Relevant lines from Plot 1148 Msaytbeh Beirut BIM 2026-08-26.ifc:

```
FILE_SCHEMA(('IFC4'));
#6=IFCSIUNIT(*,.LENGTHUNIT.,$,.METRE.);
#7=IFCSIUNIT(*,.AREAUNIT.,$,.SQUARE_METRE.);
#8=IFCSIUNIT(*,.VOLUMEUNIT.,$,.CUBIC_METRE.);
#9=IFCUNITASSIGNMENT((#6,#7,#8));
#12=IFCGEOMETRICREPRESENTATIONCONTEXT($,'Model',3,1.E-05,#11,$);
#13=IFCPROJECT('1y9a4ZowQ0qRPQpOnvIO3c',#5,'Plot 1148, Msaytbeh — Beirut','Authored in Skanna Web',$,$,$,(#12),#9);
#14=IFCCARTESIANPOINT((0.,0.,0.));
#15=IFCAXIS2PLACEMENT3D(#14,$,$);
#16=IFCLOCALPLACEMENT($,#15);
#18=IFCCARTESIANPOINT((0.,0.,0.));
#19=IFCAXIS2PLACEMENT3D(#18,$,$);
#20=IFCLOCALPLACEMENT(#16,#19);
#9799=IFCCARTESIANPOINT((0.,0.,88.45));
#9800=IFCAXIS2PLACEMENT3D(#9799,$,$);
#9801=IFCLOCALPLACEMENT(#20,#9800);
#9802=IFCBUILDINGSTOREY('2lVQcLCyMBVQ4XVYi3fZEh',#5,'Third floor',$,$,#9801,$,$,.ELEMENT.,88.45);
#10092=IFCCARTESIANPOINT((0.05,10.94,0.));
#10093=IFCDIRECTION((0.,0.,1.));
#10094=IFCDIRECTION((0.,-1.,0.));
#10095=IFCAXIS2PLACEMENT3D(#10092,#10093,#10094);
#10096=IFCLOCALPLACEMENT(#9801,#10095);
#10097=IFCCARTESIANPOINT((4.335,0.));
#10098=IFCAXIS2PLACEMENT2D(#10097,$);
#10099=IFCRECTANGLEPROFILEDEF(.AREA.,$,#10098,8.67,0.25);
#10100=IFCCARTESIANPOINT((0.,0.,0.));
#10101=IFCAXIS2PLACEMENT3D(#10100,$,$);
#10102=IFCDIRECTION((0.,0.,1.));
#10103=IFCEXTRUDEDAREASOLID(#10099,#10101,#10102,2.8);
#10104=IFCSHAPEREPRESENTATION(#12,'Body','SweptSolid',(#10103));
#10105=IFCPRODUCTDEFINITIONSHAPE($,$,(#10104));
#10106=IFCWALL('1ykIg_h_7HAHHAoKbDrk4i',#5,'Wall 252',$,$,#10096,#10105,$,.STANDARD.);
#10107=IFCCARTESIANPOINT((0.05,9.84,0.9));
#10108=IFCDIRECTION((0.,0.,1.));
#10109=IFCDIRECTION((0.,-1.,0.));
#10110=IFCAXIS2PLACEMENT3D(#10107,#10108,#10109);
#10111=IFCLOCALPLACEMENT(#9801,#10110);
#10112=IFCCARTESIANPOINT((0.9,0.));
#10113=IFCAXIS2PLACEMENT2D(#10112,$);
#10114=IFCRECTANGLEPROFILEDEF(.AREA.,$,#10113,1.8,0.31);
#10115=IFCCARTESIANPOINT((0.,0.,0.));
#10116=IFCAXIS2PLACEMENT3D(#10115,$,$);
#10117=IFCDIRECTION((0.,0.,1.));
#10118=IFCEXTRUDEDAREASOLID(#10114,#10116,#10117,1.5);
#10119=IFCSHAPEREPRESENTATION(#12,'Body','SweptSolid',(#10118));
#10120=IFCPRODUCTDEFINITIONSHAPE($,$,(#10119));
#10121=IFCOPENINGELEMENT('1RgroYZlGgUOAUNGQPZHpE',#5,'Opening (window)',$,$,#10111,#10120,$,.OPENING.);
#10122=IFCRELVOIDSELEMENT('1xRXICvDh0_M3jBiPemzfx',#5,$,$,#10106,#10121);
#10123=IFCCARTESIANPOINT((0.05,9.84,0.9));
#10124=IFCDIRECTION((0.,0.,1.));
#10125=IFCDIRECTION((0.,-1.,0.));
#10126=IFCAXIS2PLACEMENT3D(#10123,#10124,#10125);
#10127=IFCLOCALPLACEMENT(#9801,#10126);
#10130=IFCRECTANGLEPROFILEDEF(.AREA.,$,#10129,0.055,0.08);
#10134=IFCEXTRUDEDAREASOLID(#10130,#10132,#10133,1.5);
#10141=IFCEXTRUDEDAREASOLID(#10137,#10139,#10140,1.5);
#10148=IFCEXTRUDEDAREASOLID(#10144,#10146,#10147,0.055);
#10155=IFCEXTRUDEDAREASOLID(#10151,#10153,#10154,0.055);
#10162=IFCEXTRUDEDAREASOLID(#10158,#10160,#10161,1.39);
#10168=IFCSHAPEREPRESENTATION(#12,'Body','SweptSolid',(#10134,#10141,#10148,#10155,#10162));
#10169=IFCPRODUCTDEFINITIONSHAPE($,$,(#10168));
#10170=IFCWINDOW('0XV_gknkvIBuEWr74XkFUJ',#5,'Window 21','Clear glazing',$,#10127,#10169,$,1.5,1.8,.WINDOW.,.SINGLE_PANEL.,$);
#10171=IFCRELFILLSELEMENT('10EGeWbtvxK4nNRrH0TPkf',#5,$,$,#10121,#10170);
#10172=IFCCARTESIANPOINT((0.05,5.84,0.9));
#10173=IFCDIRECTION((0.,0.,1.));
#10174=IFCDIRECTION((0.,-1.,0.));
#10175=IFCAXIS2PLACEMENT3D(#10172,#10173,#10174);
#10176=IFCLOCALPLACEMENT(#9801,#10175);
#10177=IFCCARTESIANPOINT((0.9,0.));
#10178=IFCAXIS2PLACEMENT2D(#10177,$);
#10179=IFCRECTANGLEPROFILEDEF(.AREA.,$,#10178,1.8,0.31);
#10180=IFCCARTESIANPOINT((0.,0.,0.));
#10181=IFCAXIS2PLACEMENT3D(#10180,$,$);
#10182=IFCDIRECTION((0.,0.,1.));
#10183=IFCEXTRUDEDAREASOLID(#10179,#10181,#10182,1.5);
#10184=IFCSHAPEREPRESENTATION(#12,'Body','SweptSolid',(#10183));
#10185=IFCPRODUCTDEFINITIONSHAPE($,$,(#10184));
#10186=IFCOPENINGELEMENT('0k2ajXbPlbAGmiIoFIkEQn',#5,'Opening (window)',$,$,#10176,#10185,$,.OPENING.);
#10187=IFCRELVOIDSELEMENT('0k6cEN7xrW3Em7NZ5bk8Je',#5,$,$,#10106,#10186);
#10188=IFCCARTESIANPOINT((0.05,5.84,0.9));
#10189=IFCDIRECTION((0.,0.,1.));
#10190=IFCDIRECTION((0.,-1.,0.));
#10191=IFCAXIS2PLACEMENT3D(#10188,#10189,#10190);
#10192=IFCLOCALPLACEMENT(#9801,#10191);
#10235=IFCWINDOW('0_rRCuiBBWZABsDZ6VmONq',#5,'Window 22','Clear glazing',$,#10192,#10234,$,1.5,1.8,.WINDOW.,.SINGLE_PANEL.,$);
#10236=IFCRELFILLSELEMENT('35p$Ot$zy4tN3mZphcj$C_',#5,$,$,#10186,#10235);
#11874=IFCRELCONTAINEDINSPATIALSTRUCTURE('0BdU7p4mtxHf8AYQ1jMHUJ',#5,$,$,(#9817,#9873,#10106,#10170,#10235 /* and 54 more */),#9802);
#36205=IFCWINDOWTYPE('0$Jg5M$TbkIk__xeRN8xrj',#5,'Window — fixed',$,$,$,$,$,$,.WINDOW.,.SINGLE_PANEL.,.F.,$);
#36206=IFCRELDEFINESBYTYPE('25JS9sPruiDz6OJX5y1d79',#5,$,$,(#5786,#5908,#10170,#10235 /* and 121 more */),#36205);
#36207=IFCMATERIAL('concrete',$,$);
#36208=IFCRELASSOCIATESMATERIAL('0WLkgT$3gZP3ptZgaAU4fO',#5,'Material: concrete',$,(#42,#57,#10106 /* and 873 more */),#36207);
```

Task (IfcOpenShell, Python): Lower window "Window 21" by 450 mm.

```python
import numpy as np
import ifcopenshell
import ifcopenshell.api.geometry
import ifcopenshell.util.placement
import ifcopenshell.util.unit

model = ifcopenshell.open("Plot 1148 Msaytbeh Beirut BIM 2026-08-26.ifc")
unit_scale = ifcopenshell.util.unit.calculate_unit_scale(model)

window = model.by_id(10170)
opening = window.FillsVoids[0].RelatingOpeningElement
dz = -0.45 / unit_scale

shift = np.array([0.0, 0.0, dz])
# The window is not placed relative to its opening, so move both.
for product in (opening, window):
    matrix = ifcopenshell.util.placement.get_local_placement(product.ObjectPlacement)
    matrix[:3, 3] += shift
    ifcopenshell.api.geometry.edit_object_placement(model, product=product, matrix=matrix, is_si=False)

print(f"moved by {dz * unit_scale:+.3f} m")

model.write("Plot 1148 Msaytbeh Beirut BIM 2026-08-26_v2.ifc")
```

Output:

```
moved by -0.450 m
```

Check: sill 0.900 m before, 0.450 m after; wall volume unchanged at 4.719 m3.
